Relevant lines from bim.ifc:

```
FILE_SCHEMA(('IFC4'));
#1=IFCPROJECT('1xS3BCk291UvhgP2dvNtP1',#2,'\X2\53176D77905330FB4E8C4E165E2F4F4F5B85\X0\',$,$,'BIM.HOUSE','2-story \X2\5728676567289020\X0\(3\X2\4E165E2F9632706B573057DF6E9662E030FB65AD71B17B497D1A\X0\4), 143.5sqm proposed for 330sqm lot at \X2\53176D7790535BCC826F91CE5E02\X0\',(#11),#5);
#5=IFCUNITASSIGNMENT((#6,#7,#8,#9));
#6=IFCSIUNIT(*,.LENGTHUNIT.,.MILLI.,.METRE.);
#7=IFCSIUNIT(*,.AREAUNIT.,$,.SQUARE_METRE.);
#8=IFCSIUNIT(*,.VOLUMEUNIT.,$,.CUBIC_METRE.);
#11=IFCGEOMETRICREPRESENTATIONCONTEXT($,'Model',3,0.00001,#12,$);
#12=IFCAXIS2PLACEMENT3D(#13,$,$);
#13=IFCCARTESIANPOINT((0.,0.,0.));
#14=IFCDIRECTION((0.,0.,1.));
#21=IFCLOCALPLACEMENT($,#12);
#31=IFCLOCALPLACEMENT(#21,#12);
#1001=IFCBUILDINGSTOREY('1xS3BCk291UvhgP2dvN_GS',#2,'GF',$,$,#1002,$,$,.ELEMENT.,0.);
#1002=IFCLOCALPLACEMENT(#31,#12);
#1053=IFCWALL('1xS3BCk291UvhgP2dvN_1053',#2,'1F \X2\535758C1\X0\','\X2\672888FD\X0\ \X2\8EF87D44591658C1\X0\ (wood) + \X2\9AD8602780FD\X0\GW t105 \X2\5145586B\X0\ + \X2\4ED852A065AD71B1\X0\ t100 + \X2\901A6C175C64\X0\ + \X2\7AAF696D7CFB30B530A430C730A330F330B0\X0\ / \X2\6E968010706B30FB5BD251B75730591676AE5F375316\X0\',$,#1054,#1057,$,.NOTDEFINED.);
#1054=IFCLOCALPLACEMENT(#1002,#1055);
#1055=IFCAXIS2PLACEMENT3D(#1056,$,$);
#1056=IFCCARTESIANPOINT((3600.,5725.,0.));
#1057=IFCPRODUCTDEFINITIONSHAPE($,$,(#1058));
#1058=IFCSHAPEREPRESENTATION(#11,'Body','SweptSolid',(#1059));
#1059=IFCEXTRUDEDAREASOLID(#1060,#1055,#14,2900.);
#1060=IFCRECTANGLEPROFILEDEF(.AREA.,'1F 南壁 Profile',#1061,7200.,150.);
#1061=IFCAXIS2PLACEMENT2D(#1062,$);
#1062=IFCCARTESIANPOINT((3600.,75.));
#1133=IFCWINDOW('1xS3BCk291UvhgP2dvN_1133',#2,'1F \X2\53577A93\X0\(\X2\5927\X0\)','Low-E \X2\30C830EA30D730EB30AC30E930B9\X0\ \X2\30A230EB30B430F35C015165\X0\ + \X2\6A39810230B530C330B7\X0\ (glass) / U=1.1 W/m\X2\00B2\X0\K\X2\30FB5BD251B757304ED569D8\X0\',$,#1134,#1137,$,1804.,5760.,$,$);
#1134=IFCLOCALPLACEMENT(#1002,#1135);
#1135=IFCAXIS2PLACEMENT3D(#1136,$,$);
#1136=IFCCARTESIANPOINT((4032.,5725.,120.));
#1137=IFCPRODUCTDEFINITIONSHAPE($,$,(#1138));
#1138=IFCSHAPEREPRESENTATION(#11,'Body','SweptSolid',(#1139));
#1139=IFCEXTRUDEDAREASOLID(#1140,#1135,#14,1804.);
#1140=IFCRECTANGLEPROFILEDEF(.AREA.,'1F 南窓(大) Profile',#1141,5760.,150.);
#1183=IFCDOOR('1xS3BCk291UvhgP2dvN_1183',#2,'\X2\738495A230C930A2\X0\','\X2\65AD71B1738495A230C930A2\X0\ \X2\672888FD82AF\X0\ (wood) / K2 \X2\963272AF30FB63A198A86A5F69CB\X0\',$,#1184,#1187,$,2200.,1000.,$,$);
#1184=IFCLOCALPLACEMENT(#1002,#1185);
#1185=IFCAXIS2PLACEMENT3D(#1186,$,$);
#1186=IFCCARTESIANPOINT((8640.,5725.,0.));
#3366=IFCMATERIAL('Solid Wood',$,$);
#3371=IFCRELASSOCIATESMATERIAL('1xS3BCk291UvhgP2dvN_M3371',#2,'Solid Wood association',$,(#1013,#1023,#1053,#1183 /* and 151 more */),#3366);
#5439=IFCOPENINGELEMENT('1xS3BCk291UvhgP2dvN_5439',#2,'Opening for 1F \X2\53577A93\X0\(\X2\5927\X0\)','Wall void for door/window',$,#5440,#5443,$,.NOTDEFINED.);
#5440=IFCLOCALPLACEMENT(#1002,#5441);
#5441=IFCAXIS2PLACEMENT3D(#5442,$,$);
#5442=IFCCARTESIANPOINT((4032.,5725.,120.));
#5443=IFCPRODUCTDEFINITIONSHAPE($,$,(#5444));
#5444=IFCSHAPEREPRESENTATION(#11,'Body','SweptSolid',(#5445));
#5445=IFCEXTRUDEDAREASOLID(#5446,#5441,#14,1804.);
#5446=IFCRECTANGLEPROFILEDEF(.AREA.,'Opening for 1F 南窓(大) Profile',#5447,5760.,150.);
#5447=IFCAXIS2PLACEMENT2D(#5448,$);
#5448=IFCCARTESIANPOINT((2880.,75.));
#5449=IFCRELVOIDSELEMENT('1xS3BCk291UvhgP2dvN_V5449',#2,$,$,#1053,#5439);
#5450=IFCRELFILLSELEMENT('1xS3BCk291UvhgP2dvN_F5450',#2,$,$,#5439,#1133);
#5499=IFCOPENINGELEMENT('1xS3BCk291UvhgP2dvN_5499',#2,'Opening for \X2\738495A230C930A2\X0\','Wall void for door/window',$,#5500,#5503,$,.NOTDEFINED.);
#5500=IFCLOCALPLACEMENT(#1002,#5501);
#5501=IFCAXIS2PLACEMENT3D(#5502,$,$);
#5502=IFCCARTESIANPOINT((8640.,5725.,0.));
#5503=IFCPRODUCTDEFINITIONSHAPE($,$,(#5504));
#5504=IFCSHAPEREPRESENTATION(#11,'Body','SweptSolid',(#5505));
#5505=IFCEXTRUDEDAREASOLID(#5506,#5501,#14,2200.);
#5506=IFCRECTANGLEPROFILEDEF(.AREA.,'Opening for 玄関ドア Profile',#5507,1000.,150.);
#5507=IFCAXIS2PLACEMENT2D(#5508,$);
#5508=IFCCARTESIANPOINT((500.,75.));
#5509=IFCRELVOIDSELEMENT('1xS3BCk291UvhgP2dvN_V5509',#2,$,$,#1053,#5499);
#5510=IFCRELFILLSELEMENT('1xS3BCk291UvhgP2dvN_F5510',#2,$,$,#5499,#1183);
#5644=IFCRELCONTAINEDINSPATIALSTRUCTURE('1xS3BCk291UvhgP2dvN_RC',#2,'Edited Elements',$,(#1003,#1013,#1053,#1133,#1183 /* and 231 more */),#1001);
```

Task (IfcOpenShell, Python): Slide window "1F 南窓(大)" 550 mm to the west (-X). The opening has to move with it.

```python
import ifcopenshell
import ifcopenshell.api.geometry
import ifcopenshell.util.placement
import ifcopenshell.util.unit

model = ifcopenshell.open("bim.ifc")
unit_scale = ifcopenshell.util.unit.calculate_unit_scale(model)

window = model.by_id(1133)
opening = window.FillsVoids[0].RelatingOpeningElement
wall = opening.VoidsElements[0].RelatingBuildingElement

wall_matrix = ifcopenshell.util.placement.get_local_placement(wall.ObjectPlacement)
shift = wall_matrix[:3, 0] * -0.55 / unit_scale
before = ifcopenshell.util.placement.get_local_placement(window.ObjectPlacement)[:3, 3].copy()

# The window is not placed relative to its opening, so move both.
for product in (opening, window):
    matrix = ifcopenshell.util.placement.get_local_placement(product.ObjectPlacement)
    matrix[:3, 3] += shift
    ifcopenshell.api.geometry.edit_object_placement(model, product=product, matrix=matrix, is_si=False)

after = ifcopenshell.util.placement.get_local_placement(window.ObjectPlacement)[:3, 3]
print("window moved by", (after - before).round(3) + 0.0)

model.write("bim-out.ifc")
```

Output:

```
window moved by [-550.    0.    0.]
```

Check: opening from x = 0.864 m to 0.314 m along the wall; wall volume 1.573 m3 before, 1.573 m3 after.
